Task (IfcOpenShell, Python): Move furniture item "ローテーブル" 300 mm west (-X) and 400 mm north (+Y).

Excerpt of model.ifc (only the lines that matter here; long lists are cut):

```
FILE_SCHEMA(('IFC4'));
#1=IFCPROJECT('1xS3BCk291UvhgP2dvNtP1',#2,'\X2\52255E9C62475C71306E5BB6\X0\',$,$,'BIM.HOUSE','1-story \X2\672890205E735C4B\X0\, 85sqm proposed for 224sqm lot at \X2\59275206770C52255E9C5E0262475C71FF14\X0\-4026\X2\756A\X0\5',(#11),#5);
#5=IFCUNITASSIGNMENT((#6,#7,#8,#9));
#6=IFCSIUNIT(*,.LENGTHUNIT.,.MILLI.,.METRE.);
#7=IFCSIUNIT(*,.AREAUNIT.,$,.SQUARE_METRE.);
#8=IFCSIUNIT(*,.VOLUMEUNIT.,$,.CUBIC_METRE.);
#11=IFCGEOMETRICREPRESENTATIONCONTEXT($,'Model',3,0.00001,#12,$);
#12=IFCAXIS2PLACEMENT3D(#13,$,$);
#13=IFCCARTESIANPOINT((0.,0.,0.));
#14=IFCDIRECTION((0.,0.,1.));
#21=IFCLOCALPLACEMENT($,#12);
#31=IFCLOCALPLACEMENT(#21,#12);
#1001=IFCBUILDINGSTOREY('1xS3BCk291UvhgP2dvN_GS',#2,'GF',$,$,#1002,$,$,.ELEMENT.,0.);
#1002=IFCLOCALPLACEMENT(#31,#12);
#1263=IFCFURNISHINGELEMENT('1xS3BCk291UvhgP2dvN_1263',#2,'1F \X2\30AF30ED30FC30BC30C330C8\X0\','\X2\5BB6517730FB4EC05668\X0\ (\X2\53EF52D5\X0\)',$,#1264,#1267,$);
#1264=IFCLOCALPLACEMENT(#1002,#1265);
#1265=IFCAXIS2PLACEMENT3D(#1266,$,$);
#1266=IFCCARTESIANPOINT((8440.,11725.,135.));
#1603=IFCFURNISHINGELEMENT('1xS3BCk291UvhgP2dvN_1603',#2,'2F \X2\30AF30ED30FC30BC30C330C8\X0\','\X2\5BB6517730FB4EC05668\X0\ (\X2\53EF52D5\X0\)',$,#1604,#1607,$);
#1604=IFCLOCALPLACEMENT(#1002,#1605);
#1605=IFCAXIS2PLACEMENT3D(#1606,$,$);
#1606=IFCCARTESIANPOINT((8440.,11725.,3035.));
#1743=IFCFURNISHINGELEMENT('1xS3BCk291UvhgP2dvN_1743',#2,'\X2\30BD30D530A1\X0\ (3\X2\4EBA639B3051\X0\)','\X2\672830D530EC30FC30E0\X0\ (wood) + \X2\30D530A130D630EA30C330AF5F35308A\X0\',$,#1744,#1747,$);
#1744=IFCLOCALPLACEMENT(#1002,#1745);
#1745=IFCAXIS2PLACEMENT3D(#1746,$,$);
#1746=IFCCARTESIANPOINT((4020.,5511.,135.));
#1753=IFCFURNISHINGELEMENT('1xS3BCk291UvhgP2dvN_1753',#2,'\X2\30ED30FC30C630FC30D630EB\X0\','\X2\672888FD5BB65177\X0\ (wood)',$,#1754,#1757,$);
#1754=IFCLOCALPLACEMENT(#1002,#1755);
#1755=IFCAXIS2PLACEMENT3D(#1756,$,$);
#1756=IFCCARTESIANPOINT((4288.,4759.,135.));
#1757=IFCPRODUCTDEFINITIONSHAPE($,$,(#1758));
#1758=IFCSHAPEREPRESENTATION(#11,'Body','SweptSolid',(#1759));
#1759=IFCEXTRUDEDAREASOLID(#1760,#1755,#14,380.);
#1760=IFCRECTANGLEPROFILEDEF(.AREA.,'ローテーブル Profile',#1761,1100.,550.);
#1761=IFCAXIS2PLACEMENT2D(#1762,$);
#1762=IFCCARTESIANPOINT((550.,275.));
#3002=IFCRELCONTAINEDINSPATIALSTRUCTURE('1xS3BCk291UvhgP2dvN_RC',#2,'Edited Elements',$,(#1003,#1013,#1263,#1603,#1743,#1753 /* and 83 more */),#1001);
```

```python
import ifcopenshell
import ifcopenshell.api.geometry
import ifcopenshell.util.placement
import ifcopenshell.util.unit

model = ifcopenshell.open("model.ifc")
unit_scale = ifcopenshell.util.unit.calculate_unit_scale(model)

item = model.by_guid("1xS3BCk291UvhgP2dvN_1753")
matrix = ifcopenshell.util.placement.get_local_placement(item.ObjectPlacement)
matrix[0, 3] -= 0.3 / unit_scale
matrix[1, 3] += 0.4 / unit_scale
ifcopenshell.api.geometry.edit_object_placement(model, product=item, matrix=matrix, is_si=False)

print(ifcopenshell.util.placement.get_local_placement(item.ObjectPlacement).round(3) + 0.0)

model.write("model_rev.ifc")
```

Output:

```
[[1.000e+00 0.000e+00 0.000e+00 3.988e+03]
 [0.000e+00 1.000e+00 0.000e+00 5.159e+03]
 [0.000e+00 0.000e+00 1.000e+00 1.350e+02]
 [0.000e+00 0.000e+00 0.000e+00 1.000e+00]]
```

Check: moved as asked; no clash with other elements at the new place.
